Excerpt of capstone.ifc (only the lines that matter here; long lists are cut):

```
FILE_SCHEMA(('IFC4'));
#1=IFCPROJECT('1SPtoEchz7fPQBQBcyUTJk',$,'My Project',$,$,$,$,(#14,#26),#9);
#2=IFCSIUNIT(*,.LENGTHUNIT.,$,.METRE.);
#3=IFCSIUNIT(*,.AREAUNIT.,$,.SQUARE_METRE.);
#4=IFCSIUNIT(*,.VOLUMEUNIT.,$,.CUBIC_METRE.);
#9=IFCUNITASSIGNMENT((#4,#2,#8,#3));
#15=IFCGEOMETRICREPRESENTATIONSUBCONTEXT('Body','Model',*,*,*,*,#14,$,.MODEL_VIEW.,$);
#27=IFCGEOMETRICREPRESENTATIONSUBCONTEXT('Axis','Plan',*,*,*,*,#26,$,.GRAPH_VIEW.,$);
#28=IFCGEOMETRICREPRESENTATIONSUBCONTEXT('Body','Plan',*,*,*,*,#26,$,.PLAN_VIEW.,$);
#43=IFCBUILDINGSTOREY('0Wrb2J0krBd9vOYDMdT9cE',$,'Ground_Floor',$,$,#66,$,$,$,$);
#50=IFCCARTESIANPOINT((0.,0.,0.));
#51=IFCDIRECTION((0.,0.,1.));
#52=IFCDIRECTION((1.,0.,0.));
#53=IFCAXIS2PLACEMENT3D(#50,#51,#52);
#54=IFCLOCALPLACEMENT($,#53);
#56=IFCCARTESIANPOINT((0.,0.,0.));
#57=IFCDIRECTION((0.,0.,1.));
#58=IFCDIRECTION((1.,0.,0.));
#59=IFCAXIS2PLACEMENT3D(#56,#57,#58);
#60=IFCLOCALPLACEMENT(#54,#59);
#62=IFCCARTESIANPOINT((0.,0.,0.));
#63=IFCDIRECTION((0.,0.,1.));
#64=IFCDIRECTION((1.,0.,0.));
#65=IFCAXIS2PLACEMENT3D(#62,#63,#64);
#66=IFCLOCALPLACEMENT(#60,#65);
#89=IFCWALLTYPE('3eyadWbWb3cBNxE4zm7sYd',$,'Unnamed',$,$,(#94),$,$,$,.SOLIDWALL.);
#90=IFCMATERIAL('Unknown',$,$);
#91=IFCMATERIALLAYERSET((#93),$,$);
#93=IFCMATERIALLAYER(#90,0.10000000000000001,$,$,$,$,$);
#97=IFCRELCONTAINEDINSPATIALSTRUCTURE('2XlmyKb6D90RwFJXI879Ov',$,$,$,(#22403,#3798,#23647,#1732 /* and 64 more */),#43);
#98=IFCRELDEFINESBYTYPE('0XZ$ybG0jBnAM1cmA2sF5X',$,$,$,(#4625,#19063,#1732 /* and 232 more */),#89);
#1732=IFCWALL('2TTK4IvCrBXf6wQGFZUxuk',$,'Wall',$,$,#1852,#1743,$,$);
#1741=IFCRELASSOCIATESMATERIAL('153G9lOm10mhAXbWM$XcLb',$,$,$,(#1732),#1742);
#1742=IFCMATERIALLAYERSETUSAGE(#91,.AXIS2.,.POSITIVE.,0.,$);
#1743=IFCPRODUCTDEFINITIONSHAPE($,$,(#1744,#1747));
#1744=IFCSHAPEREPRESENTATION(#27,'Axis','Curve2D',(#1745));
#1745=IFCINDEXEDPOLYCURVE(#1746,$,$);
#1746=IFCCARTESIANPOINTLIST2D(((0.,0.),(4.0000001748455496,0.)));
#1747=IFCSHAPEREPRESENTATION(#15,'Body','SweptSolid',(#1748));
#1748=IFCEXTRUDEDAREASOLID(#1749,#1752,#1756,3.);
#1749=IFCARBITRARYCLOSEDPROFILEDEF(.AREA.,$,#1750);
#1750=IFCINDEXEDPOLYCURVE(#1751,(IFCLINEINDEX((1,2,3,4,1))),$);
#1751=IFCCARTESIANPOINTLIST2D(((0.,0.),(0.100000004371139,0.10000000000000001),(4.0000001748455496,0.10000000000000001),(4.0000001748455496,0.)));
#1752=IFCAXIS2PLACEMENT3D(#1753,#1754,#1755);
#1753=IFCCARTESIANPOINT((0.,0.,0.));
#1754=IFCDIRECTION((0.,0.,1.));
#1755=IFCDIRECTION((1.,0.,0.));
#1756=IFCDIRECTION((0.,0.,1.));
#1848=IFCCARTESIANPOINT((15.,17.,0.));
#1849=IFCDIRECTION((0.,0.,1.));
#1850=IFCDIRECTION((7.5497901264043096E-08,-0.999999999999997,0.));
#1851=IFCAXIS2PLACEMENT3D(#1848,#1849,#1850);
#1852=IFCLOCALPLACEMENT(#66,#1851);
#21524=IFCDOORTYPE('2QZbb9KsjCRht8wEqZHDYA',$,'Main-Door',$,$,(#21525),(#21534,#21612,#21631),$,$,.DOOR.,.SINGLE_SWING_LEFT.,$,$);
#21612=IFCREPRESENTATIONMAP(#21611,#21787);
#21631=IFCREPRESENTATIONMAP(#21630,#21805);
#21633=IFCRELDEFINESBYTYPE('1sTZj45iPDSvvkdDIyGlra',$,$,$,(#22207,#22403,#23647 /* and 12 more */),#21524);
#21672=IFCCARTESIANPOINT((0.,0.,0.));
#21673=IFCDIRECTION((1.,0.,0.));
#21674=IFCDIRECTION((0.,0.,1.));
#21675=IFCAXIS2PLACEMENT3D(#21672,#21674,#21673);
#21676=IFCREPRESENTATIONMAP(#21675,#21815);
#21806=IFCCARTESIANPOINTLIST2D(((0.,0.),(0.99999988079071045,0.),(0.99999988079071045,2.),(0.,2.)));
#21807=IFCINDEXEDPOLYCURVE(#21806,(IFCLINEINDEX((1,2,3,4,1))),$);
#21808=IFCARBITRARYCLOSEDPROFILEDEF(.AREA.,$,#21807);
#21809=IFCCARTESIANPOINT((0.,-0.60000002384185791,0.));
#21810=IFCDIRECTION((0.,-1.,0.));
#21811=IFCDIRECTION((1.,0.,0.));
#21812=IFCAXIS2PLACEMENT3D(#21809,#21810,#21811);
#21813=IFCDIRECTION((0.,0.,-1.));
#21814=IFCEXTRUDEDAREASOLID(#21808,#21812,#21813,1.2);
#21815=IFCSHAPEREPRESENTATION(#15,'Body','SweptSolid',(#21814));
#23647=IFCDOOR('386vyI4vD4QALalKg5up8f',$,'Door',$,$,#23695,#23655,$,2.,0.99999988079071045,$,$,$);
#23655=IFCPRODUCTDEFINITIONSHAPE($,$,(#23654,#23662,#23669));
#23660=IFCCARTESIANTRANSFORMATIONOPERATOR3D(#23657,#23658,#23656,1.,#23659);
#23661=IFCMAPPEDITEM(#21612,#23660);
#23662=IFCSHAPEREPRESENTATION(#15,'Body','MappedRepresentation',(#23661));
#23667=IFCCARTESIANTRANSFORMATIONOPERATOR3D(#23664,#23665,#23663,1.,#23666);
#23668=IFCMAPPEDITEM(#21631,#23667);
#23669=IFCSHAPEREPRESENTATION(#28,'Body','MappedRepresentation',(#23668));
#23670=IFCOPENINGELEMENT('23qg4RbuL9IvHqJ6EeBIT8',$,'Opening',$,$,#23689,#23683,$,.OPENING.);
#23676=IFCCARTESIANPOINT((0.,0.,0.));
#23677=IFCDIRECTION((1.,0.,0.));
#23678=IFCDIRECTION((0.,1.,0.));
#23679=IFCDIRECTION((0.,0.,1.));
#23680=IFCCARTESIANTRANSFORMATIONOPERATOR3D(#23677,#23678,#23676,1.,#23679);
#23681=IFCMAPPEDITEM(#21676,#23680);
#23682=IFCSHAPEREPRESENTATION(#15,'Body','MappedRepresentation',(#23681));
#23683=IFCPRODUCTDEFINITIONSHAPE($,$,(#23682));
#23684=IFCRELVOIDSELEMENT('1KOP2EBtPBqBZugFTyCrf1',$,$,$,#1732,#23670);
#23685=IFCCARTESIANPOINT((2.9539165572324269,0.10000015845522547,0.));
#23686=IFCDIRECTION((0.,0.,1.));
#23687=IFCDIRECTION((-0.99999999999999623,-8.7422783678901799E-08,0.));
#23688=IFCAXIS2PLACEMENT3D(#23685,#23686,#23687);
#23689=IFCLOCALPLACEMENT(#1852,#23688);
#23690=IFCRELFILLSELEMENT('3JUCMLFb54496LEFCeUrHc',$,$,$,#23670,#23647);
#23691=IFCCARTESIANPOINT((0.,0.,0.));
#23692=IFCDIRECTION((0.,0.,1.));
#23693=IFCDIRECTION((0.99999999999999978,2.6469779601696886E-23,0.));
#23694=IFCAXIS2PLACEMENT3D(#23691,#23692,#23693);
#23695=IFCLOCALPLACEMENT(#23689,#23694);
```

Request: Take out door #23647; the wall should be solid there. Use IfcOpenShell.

```python
import ifcopenshell
import ifcopenshell.api.feature
import ifcopenshell.api.root
import ifcopenshell.geom
import ifcopenshell.util.shape

model = ifcopenshell.open("capstone.ifc")
settings = ifcopenshell.geom.settings()


def volume(element):
    """Net volume in cubic metres, openings subtracted."""
    shape = ifcopenshell.geom.create_shape(settings, element)
    return ifcopenshell.util.shape.get_volume(shape.geometry)


door = model.by_guid("386vyI4vD4QALalKg5up8f")
opening = door.FillsVoids[0].RelatingOpeningElement
wall = opening.VoidsElements[0].RelatingBuildingElement
before = volume(wall)

ifcopenshell.api.root.remove_product(model, product=door)
ifcopenshell.api.feature.remove_feature(model, feature=opening)

after = volume(wall)

print(f"wall volume {before:.3f} -> {after:.3f} m3")

model.write("capstone-out.ifc")
```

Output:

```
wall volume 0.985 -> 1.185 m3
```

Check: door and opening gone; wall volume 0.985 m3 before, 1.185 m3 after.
